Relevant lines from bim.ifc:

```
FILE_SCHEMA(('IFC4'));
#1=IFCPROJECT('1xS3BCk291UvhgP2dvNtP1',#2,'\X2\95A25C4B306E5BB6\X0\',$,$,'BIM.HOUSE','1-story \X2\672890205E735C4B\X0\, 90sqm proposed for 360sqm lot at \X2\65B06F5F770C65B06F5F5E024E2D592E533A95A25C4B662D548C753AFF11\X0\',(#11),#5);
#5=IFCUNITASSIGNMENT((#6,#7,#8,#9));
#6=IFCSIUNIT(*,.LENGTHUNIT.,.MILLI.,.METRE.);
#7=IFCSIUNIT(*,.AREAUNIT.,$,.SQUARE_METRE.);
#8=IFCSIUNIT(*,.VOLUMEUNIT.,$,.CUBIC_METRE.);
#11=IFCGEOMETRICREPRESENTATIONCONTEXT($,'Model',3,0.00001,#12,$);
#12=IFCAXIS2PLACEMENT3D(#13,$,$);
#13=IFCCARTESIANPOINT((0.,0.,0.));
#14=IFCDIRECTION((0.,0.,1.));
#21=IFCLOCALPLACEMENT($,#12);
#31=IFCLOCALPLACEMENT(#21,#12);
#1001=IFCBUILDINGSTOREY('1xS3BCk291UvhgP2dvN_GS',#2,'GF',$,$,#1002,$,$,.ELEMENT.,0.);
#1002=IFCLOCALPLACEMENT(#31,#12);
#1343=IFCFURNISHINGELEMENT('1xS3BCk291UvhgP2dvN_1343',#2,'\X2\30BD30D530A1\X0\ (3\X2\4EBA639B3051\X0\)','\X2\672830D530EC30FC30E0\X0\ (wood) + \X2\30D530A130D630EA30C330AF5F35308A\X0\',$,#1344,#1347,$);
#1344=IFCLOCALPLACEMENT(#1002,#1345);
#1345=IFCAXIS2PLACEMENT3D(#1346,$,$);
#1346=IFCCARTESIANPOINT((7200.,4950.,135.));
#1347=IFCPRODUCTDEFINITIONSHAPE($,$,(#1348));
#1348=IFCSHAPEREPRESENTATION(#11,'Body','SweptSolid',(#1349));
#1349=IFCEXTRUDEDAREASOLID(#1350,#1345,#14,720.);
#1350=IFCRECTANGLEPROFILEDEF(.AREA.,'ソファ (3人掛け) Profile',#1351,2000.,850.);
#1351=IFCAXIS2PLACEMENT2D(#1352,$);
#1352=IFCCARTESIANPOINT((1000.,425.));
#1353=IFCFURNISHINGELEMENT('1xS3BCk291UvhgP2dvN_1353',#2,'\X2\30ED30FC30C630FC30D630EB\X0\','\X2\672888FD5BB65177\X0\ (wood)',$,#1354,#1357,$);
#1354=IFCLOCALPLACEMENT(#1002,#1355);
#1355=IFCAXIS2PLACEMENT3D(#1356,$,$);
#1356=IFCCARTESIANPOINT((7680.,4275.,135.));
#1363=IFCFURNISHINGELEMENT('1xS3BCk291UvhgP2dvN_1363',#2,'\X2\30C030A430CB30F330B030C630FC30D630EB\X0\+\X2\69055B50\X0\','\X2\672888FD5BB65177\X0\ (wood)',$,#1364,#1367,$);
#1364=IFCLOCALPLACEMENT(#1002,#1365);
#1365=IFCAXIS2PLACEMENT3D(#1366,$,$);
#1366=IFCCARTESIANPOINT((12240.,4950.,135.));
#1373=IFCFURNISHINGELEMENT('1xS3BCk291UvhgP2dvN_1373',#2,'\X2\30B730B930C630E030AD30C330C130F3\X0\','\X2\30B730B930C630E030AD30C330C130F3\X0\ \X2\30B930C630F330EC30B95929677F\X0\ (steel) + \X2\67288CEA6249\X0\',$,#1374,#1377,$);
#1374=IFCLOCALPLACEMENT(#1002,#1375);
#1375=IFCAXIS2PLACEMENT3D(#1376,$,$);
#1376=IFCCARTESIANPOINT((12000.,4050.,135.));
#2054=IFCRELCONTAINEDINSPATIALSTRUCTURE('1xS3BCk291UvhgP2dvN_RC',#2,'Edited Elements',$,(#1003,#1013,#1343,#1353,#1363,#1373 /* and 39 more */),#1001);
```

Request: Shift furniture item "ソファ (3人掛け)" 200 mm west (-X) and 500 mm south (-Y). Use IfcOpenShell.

```python
import ifcopenshell
import ifcopenshell.api.geometry
import ifcopenshell.util.placement
import ifcopenshell.util.unit

model = ifcopenshell.open("bim.ifc")
unit_scale = ifcopenshell.util.unit.calculate_unit_scale(model)

item = model.by_guid("1xS3BCk291UvhgP2dvN_1343")
matrix = ifcopenshell.util.placement.get_local_placement(item.ObjectPlacement)
matrix[0, 3] -= 0.2 / unit_scale
matrix[1, 3] -= 0.5 / unit_scale
ifcopenshell.api.geometry.edit_object_placement(model, product=item, matrix=matrix, is_si=False)

print(ifcopenshell.util.placement.get_local_placement(item.ObjectPlacement).round(3) + 0.0)

model.write("bim-out.ifc")
```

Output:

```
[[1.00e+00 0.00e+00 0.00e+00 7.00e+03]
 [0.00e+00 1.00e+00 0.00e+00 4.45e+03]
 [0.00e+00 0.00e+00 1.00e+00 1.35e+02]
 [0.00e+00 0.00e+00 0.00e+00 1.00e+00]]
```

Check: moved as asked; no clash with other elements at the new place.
